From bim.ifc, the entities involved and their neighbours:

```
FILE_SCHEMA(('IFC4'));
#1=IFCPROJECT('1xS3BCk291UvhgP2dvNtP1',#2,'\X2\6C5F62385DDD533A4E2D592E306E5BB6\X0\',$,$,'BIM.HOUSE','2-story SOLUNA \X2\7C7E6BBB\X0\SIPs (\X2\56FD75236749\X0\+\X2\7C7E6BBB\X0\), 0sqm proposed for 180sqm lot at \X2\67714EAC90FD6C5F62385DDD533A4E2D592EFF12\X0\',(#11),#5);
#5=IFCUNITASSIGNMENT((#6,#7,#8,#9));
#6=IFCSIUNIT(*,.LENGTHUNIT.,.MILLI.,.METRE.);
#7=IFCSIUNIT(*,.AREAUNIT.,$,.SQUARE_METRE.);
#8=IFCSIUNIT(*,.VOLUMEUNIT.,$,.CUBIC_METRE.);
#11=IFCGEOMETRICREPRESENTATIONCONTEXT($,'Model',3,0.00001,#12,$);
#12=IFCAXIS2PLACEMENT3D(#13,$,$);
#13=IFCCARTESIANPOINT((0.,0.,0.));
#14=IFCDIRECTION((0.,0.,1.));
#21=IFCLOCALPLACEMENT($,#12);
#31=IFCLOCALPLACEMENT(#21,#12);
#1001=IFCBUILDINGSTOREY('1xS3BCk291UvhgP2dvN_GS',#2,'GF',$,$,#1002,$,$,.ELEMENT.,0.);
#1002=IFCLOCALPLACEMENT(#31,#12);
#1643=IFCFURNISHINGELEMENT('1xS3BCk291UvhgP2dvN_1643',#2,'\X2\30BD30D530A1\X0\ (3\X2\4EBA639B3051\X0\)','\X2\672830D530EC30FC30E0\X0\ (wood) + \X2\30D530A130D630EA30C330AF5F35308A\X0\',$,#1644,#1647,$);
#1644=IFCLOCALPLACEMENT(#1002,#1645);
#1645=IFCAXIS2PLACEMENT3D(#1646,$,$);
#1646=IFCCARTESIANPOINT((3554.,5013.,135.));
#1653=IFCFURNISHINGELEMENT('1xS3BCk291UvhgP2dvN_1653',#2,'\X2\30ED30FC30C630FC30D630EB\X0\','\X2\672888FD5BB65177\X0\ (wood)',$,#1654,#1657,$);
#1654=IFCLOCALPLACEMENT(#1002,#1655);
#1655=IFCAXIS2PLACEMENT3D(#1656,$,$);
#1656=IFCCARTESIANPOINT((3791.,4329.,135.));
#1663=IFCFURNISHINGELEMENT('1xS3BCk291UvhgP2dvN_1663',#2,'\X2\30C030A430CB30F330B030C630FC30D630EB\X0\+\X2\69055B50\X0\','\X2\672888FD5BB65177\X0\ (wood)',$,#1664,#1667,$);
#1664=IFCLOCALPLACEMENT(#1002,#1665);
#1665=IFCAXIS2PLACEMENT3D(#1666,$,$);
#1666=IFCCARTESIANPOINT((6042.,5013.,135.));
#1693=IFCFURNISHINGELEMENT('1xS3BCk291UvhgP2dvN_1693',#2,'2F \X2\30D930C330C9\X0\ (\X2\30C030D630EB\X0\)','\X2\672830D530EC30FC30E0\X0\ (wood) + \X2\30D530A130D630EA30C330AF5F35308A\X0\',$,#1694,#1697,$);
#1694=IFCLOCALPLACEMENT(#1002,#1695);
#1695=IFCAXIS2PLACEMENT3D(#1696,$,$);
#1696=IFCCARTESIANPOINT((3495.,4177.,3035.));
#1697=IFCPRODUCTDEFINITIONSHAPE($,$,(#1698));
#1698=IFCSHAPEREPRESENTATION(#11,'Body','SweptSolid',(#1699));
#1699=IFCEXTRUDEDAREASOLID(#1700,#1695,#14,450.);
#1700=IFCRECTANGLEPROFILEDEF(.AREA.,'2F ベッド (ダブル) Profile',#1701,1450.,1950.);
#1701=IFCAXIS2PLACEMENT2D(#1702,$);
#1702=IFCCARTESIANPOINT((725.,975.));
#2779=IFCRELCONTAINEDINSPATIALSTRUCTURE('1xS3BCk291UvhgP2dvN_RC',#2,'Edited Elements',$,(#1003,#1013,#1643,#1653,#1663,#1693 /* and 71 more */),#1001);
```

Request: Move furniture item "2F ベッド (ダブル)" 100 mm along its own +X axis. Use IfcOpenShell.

```python
import ifcopenshell
import ifcopenshell.api.geometry
import ifcopenshell.util.placement

model = ifcopenshell.open("bim.ifc")

item = model.by_guid("1xS3BCk291UvhgP2dvN_1693")
matrix = ifcopenshell.util.placement.get_local_placement(item.ObjectPlacement)
matrix[:3, 3] += matrix[:3, 0] * 100.0
ifcopenshell.api.geometry.edit_object_placement(model, product=item, matrix=matrix, is_si=False)

print(ifcopenshell.util.placement.get_local_placement(item.ObjectPlacement).round(3) + 0.0)

model.write("bim_v2.ifc")
```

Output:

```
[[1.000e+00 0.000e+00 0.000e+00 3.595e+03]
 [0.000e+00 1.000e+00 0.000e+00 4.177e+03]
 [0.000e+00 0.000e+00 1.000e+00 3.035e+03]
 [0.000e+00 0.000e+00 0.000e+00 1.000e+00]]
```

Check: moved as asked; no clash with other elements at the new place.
